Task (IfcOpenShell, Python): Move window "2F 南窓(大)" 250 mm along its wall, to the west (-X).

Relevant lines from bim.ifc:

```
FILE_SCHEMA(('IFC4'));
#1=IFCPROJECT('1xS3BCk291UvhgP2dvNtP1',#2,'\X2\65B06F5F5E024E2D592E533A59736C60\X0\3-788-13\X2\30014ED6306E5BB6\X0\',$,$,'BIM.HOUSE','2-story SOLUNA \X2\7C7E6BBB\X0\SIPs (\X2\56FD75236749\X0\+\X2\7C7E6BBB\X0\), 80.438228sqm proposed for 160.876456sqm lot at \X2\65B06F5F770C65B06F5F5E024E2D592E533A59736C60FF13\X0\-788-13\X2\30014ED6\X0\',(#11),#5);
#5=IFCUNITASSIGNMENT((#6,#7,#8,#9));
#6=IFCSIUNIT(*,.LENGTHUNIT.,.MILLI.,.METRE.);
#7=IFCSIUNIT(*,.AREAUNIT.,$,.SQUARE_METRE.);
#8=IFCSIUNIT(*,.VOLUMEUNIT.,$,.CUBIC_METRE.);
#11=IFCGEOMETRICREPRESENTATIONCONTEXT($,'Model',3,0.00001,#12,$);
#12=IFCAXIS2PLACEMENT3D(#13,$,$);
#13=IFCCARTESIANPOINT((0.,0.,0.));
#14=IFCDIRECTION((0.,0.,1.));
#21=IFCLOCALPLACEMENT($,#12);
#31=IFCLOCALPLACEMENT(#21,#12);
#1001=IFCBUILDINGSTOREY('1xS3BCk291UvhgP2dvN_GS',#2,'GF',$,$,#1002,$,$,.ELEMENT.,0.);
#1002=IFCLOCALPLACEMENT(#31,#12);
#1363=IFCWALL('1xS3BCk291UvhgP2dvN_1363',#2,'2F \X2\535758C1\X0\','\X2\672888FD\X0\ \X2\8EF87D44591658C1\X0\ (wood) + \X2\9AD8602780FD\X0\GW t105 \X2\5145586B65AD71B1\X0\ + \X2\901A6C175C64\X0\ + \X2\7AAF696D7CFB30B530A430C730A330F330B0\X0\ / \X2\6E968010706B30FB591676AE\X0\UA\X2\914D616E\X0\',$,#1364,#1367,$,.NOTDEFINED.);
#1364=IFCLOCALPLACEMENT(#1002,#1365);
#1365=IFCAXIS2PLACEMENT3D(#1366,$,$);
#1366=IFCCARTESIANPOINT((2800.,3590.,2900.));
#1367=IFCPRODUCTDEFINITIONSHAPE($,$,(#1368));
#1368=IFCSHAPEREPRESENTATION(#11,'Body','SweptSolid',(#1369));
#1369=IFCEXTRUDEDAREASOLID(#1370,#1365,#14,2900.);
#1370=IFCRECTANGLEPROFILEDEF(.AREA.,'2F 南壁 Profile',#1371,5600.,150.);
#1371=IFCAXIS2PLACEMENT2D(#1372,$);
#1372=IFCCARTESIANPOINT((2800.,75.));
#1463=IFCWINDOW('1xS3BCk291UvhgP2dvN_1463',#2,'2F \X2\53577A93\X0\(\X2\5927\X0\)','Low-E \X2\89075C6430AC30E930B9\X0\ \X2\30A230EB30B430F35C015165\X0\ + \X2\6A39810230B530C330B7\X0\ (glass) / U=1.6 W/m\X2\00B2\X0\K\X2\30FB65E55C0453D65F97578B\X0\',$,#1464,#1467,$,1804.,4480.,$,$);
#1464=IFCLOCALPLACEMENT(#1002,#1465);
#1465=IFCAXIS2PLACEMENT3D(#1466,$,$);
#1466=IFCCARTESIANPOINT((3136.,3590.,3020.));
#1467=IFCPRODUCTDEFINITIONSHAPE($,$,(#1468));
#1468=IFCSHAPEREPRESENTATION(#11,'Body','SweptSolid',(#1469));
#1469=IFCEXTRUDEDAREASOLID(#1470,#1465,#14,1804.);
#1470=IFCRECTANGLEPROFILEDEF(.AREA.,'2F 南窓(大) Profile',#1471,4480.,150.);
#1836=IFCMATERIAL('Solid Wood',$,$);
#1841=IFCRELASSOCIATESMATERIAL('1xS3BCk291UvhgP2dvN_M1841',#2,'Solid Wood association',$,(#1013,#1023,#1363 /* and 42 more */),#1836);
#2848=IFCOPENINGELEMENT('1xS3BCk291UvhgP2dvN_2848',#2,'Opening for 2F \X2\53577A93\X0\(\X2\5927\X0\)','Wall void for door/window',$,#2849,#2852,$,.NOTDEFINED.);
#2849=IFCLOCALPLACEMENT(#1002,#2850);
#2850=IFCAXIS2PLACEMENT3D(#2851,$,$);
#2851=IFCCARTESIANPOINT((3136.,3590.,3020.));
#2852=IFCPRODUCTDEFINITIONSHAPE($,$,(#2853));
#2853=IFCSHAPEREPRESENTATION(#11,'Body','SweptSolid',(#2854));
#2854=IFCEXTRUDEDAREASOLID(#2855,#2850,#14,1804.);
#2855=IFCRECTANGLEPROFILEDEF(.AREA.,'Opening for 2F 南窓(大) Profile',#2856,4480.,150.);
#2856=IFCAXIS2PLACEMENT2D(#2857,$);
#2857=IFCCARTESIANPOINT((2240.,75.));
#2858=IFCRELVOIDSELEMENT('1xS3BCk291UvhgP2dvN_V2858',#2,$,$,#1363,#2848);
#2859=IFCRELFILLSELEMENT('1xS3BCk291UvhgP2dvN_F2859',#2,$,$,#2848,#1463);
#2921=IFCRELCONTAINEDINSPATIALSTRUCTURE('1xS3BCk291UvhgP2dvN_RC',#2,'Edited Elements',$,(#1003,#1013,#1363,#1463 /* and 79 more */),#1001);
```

```python
import ifcopenshell
import ifcopenshell.api.geometry
import ifcopenshell.util.placement
import ifcopenshell.util.unit

model = ifcopenshell.open("bim.ifc")
unit_scale = ifcopenshell.util.unit.calculate_unit_scale(model)

window = model.by_guid("1xS3BCk291UvhgP2dvN_1463")
opening = window.FillsVoids[0].RelatingOpeningElement
wall = opening.VoidsElements[0].RelatingBuildingElement

wall_matrix = ifcopenshell.util.placement.get_local_placement(wall.ObjectPlacement)
shift = wall_matrix[:3, 0] * -0.25 / unit_scale
before = ifcopenshell.util.placement.get_local_placement(window.ObjectPlacement)[:3, 3].copy()

# The window is not placed relative to its opening, so move both.
for product in (opening, window):
    matrix = ifcopenshell.util.placement.get_local_placement(product.ObjectPlacement)
    matrix[:3, 3] += shift
    ifcopenshell.api.geometry.edit_object_placement(model, product=product, matrix=matrix, is_si=False)

after = ifcopenshell.util.placement.get_local_placement(window.ObjectPlacement)[:3, 3]
print("window moved by", (after - before).round(3) + 0.0)

model.write("bim_edited.ifc")
```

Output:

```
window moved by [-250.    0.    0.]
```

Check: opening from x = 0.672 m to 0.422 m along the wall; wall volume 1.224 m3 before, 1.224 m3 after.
